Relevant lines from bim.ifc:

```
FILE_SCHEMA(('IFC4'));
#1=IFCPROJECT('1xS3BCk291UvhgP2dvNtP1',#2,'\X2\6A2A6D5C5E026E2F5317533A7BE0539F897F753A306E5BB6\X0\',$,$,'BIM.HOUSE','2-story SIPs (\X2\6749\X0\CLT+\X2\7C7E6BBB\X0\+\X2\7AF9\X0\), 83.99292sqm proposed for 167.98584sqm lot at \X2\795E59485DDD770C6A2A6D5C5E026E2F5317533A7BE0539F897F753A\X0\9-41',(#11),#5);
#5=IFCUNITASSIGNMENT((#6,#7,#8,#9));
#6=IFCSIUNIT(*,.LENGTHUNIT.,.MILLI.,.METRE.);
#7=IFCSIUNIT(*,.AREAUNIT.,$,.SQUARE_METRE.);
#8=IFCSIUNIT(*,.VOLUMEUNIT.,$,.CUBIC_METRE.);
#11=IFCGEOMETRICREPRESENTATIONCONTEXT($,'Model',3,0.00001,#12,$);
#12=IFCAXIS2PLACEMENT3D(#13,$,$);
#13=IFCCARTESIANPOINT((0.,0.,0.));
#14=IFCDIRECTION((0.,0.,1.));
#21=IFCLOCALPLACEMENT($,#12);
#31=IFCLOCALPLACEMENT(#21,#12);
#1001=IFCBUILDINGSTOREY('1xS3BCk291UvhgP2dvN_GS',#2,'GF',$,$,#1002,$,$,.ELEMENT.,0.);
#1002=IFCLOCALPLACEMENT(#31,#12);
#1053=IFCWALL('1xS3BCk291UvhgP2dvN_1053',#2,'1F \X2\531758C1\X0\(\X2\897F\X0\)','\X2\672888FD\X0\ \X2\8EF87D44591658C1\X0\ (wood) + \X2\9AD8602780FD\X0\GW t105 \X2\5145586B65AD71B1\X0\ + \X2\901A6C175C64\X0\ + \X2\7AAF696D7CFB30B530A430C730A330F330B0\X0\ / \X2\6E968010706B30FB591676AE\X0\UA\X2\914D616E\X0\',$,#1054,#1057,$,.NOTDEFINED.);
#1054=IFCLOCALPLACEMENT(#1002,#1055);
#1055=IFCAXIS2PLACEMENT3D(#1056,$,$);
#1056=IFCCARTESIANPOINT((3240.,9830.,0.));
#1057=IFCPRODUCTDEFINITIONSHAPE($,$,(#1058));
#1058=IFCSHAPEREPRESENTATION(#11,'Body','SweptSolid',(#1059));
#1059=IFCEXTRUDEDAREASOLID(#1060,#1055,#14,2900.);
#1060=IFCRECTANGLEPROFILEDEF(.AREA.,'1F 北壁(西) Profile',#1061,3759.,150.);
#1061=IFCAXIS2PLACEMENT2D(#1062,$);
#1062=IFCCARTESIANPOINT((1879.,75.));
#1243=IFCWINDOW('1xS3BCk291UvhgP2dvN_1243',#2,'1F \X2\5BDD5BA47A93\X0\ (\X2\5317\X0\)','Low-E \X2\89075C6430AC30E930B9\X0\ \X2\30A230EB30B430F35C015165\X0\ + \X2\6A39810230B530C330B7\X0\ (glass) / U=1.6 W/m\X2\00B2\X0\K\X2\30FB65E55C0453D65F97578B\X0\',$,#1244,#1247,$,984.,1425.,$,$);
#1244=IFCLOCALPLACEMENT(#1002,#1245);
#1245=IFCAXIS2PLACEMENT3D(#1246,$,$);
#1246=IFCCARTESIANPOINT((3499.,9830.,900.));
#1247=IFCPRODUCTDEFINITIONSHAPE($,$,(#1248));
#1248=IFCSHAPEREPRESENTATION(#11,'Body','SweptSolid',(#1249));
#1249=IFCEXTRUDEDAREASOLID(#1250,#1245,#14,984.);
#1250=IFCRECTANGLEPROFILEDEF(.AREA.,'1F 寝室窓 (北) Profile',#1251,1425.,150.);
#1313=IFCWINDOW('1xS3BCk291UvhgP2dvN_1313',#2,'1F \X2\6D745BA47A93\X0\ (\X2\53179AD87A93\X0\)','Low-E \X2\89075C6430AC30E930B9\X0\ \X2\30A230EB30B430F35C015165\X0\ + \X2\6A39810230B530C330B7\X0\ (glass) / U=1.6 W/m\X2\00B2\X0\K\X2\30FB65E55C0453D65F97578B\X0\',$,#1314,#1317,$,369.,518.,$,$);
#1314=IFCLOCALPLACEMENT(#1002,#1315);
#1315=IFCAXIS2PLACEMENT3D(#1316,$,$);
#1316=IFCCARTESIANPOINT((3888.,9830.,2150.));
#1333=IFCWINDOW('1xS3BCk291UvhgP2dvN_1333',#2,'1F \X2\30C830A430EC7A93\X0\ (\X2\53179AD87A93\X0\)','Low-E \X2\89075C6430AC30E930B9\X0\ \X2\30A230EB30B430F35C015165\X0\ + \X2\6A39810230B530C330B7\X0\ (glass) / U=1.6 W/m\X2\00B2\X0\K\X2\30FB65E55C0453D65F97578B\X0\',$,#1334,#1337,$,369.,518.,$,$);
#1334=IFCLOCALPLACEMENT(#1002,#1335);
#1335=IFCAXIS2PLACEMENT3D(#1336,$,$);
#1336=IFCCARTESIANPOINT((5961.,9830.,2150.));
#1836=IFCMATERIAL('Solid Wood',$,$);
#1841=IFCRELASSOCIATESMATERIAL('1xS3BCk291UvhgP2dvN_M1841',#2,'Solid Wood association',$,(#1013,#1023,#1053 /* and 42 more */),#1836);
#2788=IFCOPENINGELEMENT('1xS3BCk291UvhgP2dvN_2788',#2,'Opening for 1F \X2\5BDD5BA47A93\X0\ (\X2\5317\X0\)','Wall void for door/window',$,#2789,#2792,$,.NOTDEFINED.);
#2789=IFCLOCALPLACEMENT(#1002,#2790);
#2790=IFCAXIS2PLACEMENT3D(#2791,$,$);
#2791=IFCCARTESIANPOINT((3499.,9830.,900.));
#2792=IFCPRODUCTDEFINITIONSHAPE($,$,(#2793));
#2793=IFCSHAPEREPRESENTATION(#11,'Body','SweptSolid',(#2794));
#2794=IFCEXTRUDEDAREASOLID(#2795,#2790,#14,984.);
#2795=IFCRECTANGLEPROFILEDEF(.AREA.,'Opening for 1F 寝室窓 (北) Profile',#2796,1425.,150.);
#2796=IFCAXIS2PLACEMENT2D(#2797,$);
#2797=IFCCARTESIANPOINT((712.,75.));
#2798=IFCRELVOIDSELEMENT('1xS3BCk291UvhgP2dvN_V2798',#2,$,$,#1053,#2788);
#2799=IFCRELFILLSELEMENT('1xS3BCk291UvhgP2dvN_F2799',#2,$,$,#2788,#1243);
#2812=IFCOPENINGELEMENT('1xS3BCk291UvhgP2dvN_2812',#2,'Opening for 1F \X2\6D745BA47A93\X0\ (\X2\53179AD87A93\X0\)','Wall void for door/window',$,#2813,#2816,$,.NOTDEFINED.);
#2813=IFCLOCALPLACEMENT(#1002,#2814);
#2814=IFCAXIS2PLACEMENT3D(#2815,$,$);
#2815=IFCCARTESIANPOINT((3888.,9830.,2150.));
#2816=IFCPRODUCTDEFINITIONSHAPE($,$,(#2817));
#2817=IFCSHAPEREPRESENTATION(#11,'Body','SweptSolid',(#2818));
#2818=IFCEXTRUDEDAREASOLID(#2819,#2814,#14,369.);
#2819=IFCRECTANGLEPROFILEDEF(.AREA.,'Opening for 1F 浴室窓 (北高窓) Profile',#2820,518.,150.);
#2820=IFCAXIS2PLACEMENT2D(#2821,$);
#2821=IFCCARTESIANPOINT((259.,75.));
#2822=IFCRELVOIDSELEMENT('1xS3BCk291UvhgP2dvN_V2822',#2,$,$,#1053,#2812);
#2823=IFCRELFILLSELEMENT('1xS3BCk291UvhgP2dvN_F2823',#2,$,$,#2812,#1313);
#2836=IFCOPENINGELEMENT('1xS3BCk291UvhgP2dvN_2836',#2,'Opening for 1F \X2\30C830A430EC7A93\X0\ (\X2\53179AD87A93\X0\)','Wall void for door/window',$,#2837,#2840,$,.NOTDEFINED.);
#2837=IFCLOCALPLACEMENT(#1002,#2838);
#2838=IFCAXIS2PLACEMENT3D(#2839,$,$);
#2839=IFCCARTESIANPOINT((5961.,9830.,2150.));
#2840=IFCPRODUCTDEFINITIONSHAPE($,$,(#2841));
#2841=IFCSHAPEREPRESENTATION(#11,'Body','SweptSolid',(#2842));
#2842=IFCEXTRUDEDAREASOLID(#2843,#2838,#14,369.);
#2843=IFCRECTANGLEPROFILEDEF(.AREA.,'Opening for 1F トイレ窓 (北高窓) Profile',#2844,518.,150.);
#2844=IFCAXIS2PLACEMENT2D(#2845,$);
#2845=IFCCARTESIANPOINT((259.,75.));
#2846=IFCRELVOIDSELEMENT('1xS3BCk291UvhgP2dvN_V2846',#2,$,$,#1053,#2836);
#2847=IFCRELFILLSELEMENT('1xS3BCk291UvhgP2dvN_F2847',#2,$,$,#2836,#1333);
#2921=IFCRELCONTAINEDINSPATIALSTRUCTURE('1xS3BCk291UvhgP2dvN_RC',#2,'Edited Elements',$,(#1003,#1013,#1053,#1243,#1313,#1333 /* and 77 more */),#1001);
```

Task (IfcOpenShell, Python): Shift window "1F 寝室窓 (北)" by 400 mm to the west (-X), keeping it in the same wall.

```python
import ifcopenshell
import ifcopenshell.api.geometry
import ifcopenshell.util.placement

model = ifcopenshell.open("bim.ifc")

window = model.by_guid("1xS3BCk291UvhgP2dvN_1243")
opening = window.FillsVoids[0].RelatingOpeningElement
wall = opening.VoidsElements[0].RelatingBuildingElement

wall_matrix = ifcopenshell.util.placement.get_local_placement(wall.ObjectPlacement)
shift = wall_matrix[:3, 0] * -400.0
before = ifcopenshell.util.placement.get_local_placement(window.ObjectPlacement)[:3, 3].copy()

# The window is not placed relative to its opening, so move both.
for product in (opening, window):
    matrix = ifcopenshell.util.placement.get_local_placement(product.ObjectPlacement)
    matrix[:3, 3] += shift
    ifcopenshell.api.geometry.edit_object_placement(model, product=product, matrix=matrix, is_si=False)

after = ifcopenshell.util.placement.get_local_placement(window.ObjectPlacement)[:3, 3]
print("window moved by", (after - before).round(3) + 0.0)

model.write("bim_v2.ifc")
```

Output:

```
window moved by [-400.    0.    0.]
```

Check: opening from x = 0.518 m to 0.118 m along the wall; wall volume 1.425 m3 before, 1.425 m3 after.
